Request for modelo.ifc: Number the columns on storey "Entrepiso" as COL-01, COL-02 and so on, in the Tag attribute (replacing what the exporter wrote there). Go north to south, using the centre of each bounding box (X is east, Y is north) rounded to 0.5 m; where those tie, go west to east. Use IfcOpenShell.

First a look at what the model holds.

```python
import ifcopenshell
import ifcopenshell.util.element
import ifcopenshell.util.placement

model = ifcopenshell.open("modelo.ifc")
print(model.schema)
storey = next(s for s in model.by_type("IfcBuildingStorey") if s.Name == "Entrepiso")
columns = [e for e in ifcopenshell.util.element.get_decomposition(storey) if e.is_a("IfcColumn")]
for e in sorted(columns, key=lambda e: e.id()):
    origin = ifcopenshell.util.placement.get_local_placement(e.ObjectPlacement)[:3, 3]
    print(e.id(), e.Tag, e.Name, origin.round(2) + 0.0, sep=" | ")
```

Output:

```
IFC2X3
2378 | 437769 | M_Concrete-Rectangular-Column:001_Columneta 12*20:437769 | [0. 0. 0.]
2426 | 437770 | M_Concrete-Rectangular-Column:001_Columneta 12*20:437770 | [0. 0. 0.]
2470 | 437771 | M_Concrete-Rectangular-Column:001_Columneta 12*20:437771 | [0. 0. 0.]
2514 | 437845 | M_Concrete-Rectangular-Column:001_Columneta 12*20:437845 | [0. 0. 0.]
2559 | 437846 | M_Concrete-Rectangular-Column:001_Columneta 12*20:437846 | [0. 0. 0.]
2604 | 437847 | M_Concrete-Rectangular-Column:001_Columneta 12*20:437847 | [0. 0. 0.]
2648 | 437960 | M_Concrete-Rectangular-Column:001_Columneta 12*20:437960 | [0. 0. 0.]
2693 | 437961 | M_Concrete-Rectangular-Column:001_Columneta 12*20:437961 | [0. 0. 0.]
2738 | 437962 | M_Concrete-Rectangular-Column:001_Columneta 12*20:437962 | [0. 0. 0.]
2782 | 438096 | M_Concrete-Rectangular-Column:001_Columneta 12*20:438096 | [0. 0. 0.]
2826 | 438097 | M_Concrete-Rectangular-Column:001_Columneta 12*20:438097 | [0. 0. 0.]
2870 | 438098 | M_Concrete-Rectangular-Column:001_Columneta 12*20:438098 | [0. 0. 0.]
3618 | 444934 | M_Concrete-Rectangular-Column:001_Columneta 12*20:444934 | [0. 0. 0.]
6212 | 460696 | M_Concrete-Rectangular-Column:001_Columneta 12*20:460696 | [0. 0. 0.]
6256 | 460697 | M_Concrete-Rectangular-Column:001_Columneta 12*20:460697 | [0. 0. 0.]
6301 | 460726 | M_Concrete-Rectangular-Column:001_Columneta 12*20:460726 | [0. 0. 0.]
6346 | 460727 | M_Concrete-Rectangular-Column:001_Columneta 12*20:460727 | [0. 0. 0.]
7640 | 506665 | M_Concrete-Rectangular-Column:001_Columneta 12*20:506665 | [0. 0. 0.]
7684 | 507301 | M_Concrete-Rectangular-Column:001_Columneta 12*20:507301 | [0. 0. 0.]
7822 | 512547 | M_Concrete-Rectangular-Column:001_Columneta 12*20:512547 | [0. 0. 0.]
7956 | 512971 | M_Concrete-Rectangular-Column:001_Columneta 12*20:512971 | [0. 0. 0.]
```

```python
import ifcopenshell
import ifcopenshell.geom
import ifcopenshell.util.element
import ifcopenshell.util.shape

model = ifcopenshell.open("modelo.ifc")
settings = ifcopenshell.geom.settings()
settings.set("use-world-coords", True)


def centre(element):
    shape = ifcopenshell.geom.create_shape(settings, element)
    return ifcopenshell.util.shape.get_bbox_centroid(shape.geometry)


storey = next(s for s in model.by_type("IfcBuildingStorey") if s.Name == "Entrepiso")
columns = [e for e in ifcopenshell.util.element.get_decomposition(storey) if e.is_a("IfcColumn")]

# Insertion points can sit at a corner or the storey origin, so sort by the geometry (in metres).
centres = {e: centre(e) for e in columns}
columns.sort(key=lambda e: (-round(centres[e][1] / 0.5), centres[e][0]))

for i, e in enumerate(columns, start=1):
    number = f"COL-{i:02d}"
    e.Tag = number
    print(e.id(), number)

model.write("modelo_edited.ifc")
```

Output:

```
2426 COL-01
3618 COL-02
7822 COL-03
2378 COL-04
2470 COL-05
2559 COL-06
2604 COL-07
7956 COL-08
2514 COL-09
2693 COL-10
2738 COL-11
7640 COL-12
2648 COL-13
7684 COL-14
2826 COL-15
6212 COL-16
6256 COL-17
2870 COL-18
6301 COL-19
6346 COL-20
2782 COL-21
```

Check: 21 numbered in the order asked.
